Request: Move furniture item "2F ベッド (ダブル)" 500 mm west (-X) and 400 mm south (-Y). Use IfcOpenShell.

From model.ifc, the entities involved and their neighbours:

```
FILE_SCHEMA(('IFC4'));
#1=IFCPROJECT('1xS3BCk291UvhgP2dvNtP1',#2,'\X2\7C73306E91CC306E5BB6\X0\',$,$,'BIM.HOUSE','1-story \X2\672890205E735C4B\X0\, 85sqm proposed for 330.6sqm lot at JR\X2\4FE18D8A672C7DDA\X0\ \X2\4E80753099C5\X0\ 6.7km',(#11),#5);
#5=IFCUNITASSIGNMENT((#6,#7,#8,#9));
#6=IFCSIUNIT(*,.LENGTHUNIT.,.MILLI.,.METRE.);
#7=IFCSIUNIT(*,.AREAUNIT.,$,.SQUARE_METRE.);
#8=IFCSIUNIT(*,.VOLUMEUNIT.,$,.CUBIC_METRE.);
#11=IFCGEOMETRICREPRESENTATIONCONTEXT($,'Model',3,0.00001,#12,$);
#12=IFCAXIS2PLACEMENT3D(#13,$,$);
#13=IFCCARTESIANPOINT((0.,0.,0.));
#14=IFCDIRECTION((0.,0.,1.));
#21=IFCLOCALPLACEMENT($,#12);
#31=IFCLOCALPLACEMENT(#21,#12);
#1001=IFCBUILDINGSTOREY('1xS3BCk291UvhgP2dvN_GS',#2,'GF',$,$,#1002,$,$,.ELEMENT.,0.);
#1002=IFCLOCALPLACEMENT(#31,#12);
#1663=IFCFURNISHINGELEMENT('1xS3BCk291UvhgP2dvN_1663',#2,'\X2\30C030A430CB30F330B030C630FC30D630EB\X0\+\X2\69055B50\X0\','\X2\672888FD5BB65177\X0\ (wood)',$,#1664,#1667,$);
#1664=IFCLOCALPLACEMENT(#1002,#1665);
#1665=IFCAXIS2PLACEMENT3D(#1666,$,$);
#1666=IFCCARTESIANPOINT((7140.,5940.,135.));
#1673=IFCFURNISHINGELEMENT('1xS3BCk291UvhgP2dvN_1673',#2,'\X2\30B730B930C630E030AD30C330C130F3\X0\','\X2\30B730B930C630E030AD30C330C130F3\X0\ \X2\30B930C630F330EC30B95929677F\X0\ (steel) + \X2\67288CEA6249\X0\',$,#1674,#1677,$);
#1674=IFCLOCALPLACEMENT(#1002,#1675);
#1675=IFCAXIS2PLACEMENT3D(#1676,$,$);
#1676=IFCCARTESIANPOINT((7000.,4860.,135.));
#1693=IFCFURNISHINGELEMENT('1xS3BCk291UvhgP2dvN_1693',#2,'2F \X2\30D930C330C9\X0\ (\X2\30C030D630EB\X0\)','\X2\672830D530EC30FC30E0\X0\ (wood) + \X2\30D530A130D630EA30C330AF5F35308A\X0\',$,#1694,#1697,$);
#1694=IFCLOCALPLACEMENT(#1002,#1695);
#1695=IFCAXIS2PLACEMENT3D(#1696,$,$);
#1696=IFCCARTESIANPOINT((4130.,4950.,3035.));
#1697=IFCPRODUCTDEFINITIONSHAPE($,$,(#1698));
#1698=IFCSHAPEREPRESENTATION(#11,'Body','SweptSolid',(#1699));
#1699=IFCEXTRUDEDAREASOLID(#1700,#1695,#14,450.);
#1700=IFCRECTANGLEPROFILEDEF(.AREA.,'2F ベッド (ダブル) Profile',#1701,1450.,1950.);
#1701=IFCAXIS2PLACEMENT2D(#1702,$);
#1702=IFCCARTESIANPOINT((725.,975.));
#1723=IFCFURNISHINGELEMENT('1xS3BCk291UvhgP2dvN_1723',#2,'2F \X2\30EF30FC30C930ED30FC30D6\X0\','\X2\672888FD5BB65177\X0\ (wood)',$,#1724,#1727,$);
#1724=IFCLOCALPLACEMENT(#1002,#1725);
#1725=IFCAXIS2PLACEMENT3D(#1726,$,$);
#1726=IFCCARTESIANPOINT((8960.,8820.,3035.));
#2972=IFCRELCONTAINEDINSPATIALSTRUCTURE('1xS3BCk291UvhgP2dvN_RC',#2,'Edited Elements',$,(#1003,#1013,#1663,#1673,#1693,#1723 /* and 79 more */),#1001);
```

```python
import ifcopenshell
import ifcopenshell.api.geometry
import ifcopenshell.util.placement
import ifcopenshell.util.unit

model = ifcopenshell.open("model.ifc")
unit_scale = ifcopenshell.util.unit.calculate_unit_scale(model)

item = model.by_guid("1xS3BCk291UvhgP2dvN_1693")
matrix = ifcopenshell.util.placement.get_local_placement(item.ObjectPlacement)
matrix[0, 3] -= 0.5 / unit_scale
matrix[1, 3] -= 0.4 / unit_scale
ifcopenshell.api.geometry.edit_object_placement(model, product=item, matrix=matrix, is_si=False)

print(ifcopenshell.util.placement.get_local_placement(item.ObjectPlacement).round(3) + 0.0)

model.write("model_rev.ifc")
```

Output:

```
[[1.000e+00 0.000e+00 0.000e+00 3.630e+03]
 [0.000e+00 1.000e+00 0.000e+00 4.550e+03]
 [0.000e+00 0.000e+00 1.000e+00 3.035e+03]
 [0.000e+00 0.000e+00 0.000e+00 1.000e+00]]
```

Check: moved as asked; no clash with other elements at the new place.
